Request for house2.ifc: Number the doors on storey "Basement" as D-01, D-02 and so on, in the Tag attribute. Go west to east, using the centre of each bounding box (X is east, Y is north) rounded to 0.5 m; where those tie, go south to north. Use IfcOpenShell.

First a look at what the model holds.

```python
import ifcopenshell
import ifcopenshell.util.element
import ifcopenshell.util.placement

model = ifcopenshell.open("house2.ifc")
print(model.schema)
storey = next(s for s in model.by_type("IfcBuildingStorey") if s.Name == "Basement")
doors = [e for e in ifcopenshell.util.element.get_decomposition(storey) if e.is_a("IfcDoor")]
for e in sorted(doors, key=lambda e: e.id()):
    origin = ifcopenshell.util.placement.get_local_placement(e.ObjectPlacement)[:3, 3]
    print(e.id(), e.Tag, e.Name, origin.round(2) + 0.0, sep=" | ")
```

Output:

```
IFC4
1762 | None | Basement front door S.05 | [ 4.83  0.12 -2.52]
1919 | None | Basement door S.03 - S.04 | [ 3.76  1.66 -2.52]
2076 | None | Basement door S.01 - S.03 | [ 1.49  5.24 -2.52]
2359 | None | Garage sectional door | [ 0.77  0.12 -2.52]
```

```python
import ifcopenshell
import ifcopenshell.geom
import ifcopenshell.util.element
import ifcopenshell.util.shape

model = ifcopenshell.open("house2.ifc")
settings = ifcopenshell.geom.settings()
settings.set("use-world-coords", True)


def centre(element):
    shape = ifcopenshell.geom.create_shape(settings, element)
    return ifcopenshell.util.shape.get_bbox_centroid(shape.geometry)


storey = next(s for s in model.by_type("IfcBuildingStorey") if s.Name == "Basement")
doors = [e for e in ifcopenshell.util.element.get_decomposition(storey) if e.is_a("IfcDoor")]

# Insertion points can sit at a corner or the storey origin, so sort by the geometry (in metres).
centres = {e: centre(e) for e in doors}
doors.sort(key=lambda e: (round(centres[e][0] / 0.5), centres[e][1]))

for i, e in enumerate(doors, start=1):
    number = f"D-{i:02d}"
    e.Tag = number
    print(e.id(), number)

model.write("house2_rev.ifc")
```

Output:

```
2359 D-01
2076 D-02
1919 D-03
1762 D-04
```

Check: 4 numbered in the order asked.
